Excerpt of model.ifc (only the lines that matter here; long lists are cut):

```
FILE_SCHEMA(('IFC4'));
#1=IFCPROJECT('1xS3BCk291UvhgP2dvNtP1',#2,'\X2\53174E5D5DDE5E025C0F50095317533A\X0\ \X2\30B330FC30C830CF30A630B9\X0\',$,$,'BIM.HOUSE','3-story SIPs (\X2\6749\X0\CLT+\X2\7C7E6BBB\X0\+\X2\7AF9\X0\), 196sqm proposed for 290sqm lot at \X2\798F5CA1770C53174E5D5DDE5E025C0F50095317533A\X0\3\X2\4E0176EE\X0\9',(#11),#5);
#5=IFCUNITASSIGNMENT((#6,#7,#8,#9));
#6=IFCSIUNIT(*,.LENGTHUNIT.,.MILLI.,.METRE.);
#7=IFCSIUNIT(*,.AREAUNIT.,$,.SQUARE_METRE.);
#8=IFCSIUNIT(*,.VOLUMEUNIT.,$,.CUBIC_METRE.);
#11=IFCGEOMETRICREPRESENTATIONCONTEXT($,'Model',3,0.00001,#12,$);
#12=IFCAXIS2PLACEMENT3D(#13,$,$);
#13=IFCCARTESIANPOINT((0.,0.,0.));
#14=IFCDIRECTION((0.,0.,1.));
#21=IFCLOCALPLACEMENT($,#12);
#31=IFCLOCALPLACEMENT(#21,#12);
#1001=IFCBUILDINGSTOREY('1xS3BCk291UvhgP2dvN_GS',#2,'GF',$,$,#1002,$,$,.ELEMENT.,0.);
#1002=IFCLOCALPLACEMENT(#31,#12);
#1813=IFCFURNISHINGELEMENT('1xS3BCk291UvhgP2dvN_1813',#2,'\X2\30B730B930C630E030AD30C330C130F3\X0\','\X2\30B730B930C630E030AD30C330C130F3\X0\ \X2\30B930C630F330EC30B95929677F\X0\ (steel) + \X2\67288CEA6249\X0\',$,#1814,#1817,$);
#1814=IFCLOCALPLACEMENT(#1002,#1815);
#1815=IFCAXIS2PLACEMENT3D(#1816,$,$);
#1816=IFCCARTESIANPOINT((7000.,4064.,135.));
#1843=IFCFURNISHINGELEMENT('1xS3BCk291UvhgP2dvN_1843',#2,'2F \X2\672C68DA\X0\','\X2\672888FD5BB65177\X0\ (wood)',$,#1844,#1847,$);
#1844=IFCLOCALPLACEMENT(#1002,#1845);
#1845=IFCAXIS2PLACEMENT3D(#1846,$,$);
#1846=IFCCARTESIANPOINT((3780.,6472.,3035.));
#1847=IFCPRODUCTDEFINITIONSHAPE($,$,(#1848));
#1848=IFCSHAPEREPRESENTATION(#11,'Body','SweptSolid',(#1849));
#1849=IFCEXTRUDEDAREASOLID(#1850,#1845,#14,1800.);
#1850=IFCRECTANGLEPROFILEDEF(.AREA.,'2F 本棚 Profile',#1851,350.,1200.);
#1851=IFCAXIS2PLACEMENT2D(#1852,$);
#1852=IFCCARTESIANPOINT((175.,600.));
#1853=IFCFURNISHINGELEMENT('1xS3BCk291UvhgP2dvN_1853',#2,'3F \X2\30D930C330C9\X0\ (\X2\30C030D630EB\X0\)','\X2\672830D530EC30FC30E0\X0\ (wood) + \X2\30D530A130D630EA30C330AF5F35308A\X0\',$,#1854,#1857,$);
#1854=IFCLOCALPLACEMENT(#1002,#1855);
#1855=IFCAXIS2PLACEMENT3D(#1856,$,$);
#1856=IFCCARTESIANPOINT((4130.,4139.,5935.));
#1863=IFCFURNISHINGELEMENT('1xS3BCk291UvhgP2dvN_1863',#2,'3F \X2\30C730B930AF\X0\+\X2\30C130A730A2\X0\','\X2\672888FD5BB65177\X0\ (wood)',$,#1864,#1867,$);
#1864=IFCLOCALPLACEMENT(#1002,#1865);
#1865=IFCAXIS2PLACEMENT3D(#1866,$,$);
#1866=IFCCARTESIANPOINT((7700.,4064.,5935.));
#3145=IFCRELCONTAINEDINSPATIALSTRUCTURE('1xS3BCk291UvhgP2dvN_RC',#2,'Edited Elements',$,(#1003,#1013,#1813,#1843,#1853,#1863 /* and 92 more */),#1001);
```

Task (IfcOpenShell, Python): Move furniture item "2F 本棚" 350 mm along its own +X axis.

```python
import ifcopenshell
import ifcopenshell.api.geometry
import ifcopenshell.util.placement

model = ifcopenshell.open("model.ifc")

item = model.by_guid("1xS3BCk291UvhgP2dvN_1843")
matrix = ifcopenshell.util.placement.get_local_placement(item.ObjectPlacement)
matrix[:3, 3] += matrix[:3, 0] * 350.0
ifcopenshell.api.geometry.edit_object_placement(model, product=item, matrix=matrix, is_si=False)

print(ifcopenshell.util.placement.get_local_placement(item.ObjectPlacement).round(3) + 0.0)

model.write("model_updated.ifc")
```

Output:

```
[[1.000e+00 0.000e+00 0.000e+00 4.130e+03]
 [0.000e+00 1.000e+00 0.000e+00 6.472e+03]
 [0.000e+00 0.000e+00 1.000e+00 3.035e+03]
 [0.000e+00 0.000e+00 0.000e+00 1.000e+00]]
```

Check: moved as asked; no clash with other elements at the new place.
